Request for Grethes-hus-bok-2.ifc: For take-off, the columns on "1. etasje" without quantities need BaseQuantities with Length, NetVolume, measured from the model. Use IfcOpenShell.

First a look at what the model holds.

```python
import ifcopenshell
import ifcopenshell.util.element
import ifcopenshell.util.unit

model = ifcopenshell.open("Grethes-hus-bok-2.ifc")
print(model.schema)
for unit_type in ("LENGTHUNIT", "AREAUNIT", "VOLUMEUNIT"):
    print(unit_type, ifcopenshell.util.unit.calculate_unit_scale(model, unit_type))
storey = next(s for s in model.by_type("IfcBuildingStorey") if s.Name == "1. etasje")
columns = [e for e in ifcopenshell.util.element.get_decomposition(storey) if e.is_a("IfcColumn")]
for e in sorted(columns, key=lambda e: e.id()):
    print(e.id(), e.is_a(), e.Name, list(ifcopenshell.util.element.get_psets(e, qtos_only=True)), sep=" | ")
```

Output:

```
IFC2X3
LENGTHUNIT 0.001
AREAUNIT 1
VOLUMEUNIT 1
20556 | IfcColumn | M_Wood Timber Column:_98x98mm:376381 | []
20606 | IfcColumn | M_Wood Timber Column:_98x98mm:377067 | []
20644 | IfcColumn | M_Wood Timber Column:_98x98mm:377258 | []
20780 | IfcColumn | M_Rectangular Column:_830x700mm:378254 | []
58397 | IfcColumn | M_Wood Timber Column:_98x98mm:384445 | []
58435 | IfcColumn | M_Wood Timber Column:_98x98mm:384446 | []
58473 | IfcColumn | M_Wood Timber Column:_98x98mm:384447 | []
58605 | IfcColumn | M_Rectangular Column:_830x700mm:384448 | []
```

```python
import ifcopenshell
import ifcopenshell.api.pset
import ifcopenshell.geom
import ifcopenshell.util.element
import ifcopenshell.util.shape
import ifcopenshell.util.unit

model = ifcopenshell.open("Grethes-hus-bok-2.ifc")
unit_scale = ifcopenshell.util.unit.calculate_unit_scale(model)
volume_scale = ifcopenshell.util.unit.calculate_unit_scale(model, "VOLUMEUNIT")
settings = ifcopenshell.geom.settings()

storey = next(s for s in model.by_type("IfcBuildingStorey") if s.Name == "1. etasje")
columns = [e for e in ifcopenshell.util.element.get_decomposition(storey) if e.is_a("IfcColumn")]

for e in sorted(columns, key=lambda e: e.id()):
    if ifcopenshell.util.element.get_psets(e, qtos_only=True, should_inherit=False):
        continue
    # Geometry comes back in metres, in the element's own axes.
    shape = ifcopenshell.geom.create_shape(settings, e)
    values = {
        "Length": ifcopenshell.util.shape.get_z(shape.geometry) / unit_scale,
        "NetVolume": ifcopenshell.util.shape.get_volume(shape.geometry) / volume_scale,
    }
    qto = ifcopenshell.api.pset.add_qto(model, product=e, name="BaseQuantities")
    ifcopenshell.api.pset.edit_qto(model, qto=qto, properties=values)
    print(e.id(), {k: round(v, 3) for k, v in values.items()})

model.write("Grethes-hus-bok-2_v2.ifc")
```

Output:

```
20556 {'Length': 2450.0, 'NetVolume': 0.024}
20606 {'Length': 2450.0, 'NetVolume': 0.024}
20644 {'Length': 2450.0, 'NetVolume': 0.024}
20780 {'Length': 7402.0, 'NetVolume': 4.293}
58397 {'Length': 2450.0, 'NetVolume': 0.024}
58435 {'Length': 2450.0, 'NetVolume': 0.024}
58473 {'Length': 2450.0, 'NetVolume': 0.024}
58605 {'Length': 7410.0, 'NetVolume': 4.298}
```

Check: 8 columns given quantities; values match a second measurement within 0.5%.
